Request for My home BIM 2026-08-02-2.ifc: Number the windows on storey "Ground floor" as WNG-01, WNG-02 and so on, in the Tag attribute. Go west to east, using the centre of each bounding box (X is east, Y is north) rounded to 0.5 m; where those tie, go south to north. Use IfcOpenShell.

First a look at what the model holds.

```python
import ifcopenshell
import ifcopenshell.util.element
import ifcopenshell.util.placement

model = ifcopenshell.open("My home BIM 2026-08-02-2.ifc")
print(model.schema)
storey = next(s for s in model.by_type("IfcBuildingStorey") if s.Name == "Ground floor")
windows = [e for e in ifcopenshell.util.element.get_decomposition(storey) if e.is_a("IfcWindow")]
for e in sorted(windows, key=lambda e: e.id()):
    origin = ifcopenshell.util.placement.get_local_placement(e.ObjectPlacement)[:3, 3]
    print(e.id(), e.Tag, e.Name, origin.round(2) + 0.0, sep=" | ")
```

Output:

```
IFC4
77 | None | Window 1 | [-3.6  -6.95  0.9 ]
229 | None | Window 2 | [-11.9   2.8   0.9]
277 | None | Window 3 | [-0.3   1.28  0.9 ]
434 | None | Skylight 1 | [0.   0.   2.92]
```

```python
import ifcopenshell
import ifcopenshell.geom
import ifcopenshell.util.element
import ifcopenshell.util.shape

model = ifcopenshell.open("My home BIM 2026-08-02-2.ifc")
settings = ifcopenshell.geom.settings()
settings.set("use-world-coords", True)


def centre(element):
    shape = ifcopenshell.geom.create_shape(settings, element)
    return ifcopenshell.util.shape.get_bbox_centroid(shape.geometry)


storey = next(s for s in model.by_type("IfcBuildingStorey") if s.Name == "Ground floor")
windows = [e for e in ifcopenshell.util.element.get_decomposition(storey) if e.is_a("IfcWindow")]

# Insertion points can sit at a corner or the storey origin, so sort by the geometry (in metres).
centres = {e: centre(e) for e in windows}
windows.sort(key=lambda e: (round(centres[e][0] / 0.5), centres[e][1]))

for i, e in enumerate(windows, start=1):
    number = f"WNG-{i:02d}"
    e.Tag = number
    print(e.id(), number)

model.write("My home BIM 2026-08-02-2_v2.ifc")
```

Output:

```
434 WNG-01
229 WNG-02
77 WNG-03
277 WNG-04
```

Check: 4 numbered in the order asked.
